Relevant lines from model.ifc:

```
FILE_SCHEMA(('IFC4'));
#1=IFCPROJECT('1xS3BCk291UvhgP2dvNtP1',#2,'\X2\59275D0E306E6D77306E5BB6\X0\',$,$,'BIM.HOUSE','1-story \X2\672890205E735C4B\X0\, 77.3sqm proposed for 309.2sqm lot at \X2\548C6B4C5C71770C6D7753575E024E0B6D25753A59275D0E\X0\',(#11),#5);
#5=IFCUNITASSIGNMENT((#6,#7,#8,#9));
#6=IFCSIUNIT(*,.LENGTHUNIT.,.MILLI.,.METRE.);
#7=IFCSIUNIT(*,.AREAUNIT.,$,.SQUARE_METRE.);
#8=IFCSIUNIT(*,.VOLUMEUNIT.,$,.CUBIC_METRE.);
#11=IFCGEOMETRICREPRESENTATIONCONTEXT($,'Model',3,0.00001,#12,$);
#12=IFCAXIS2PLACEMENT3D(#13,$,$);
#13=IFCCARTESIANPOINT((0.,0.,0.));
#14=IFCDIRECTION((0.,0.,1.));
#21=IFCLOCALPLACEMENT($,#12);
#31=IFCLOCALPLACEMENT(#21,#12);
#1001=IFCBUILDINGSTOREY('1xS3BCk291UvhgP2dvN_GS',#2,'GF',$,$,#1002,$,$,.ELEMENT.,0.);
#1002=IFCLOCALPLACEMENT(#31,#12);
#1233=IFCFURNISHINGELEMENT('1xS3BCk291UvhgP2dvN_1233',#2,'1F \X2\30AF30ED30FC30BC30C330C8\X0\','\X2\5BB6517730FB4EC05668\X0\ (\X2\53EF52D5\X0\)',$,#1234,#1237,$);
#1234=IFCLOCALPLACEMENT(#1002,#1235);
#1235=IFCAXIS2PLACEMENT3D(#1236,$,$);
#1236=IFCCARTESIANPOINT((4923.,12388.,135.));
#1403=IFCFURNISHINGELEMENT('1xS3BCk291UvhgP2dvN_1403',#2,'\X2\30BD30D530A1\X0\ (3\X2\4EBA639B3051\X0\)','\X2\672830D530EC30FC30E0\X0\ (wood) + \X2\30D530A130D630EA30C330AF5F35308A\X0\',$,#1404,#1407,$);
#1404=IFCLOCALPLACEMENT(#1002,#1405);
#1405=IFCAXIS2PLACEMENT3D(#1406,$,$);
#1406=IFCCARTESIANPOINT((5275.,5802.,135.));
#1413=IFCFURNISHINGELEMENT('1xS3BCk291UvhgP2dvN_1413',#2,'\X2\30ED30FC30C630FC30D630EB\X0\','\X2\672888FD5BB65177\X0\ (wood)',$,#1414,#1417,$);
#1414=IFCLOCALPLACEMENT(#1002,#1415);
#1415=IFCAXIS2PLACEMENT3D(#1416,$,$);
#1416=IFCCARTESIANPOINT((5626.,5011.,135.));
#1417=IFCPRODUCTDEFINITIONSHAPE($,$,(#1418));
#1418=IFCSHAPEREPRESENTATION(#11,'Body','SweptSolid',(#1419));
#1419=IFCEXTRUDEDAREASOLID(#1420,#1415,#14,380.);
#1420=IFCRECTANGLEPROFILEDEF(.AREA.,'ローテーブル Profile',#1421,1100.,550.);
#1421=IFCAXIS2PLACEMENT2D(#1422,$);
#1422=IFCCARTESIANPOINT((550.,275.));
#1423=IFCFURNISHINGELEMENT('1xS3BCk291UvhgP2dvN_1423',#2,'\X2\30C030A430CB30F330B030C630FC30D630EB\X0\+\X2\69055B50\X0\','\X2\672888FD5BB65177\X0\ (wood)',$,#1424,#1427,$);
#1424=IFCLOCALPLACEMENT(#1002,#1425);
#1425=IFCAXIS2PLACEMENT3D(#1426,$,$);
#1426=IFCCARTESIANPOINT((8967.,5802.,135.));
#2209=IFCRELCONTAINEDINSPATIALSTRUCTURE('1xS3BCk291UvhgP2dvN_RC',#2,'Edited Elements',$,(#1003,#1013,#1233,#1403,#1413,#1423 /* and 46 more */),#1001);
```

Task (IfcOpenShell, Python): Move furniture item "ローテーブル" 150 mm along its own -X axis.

```python
import ifcopenshell
import ifcopenshell.api.geometry
import ifcopenshell.util.placement

model = ifcopenshell.open("model.ifc")

item = model.by_guid("1xS3BCk291UvhgP2dvN_1413")
matrix = ifcopenshell.util.placement.get_local_placement(item.ObjectPlacement)
matrix[:3, 3] -= matrix[:3, 0] * 150.0
ifcopenshell.api.geometry.edit_object_placement(model, product=item, matrix=matrix, is_si=False)

print(ifcopenshell.util.placement.get_local_placement(item.ObjectPlacement).round(3) + 0.0)

model.write("model_updated.ifc")
```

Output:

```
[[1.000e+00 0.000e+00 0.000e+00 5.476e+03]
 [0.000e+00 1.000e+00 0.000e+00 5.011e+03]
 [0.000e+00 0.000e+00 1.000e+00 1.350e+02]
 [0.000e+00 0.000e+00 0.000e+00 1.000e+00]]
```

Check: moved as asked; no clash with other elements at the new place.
